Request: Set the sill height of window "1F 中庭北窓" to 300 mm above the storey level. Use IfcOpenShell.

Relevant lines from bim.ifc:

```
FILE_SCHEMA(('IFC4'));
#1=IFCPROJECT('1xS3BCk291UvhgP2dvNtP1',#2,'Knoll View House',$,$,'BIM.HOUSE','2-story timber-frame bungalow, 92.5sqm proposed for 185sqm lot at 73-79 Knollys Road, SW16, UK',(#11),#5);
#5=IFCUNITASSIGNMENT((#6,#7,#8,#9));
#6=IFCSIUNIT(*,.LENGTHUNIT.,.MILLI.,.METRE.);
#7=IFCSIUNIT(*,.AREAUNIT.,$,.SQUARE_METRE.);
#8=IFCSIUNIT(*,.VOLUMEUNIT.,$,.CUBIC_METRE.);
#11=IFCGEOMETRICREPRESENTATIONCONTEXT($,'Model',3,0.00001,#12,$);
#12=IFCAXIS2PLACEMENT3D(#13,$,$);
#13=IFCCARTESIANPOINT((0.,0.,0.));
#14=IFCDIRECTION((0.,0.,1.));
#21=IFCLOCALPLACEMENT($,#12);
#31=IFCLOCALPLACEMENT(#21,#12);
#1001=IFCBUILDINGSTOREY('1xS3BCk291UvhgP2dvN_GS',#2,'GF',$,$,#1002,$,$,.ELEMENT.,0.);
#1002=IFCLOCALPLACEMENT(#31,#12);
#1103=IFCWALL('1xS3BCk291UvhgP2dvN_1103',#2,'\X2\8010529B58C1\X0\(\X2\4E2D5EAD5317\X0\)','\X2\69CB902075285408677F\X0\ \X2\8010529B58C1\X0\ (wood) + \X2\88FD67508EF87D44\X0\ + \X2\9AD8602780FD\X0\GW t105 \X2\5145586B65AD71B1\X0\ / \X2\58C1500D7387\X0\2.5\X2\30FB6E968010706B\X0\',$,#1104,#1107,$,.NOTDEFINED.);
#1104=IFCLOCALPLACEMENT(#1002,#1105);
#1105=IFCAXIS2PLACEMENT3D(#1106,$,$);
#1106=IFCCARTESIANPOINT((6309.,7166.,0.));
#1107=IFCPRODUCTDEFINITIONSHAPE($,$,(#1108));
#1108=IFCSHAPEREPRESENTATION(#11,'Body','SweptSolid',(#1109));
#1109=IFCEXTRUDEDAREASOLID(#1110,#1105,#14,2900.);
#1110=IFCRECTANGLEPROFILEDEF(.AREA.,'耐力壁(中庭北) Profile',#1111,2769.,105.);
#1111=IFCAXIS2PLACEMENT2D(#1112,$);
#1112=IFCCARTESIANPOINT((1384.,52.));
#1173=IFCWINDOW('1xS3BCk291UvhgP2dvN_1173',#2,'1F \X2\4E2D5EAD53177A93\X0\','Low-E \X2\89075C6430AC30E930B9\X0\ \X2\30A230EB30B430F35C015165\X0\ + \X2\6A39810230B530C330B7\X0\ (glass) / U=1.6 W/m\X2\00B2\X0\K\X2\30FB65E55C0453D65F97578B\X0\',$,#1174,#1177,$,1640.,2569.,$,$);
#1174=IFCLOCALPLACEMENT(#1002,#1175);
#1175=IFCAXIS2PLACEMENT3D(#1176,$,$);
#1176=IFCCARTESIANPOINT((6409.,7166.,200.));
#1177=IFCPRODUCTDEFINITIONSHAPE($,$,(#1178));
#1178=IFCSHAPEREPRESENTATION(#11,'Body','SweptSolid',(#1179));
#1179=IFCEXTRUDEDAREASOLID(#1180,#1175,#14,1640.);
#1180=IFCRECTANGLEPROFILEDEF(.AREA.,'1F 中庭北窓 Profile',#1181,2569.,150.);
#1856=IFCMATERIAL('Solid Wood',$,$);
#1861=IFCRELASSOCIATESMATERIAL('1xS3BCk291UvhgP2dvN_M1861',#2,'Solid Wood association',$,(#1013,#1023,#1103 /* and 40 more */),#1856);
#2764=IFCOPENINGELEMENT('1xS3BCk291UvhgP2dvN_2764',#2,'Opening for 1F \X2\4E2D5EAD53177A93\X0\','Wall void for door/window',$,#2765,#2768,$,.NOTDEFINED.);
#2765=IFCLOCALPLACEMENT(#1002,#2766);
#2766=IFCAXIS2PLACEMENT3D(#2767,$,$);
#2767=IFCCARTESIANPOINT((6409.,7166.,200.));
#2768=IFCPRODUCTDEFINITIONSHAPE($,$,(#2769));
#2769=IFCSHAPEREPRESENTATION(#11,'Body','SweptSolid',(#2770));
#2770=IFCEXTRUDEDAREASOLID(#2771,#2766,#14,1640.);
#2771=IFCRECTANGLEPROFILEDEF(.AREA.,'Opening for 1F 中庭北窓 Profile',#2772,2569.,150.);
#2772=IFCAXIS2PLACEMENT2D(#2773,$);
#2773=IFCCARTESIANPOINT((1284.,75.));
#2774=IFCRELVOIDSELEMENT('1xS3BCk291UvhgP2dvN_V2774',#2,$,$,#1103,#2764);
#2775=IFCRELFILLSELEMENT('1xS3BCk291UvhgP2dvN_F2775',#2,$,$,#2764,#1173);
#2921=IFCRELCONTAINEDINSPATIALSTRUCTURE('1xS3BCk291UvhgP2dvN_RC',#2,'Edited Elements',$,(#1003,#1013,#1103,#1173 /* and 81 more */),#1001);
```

```python
import numpy as np
import ifcopenshell
import ifcopenshell.api.geometry
import ifcopenshell.geom
import ifcopenshell.util.element
import ifcopenshell.util.placement
import ifcopenshell.util.shape
import ifcopenshell.util.unit

model = ifcopenshell.open("bim.ifc")
unit_scale = ifcopenshell.util.unit.calculate_unit_scale(model)

window = model.by_guid("1xS3BCk291UvhgP2dvN_1173")
opening = window.FillsVoids[0].RelatingOpeningElement
storey = ifcopenshell.util.element.get_container(window, ifc_class="IfcBuildingStorey")
level = ifcopenshell.util.placement.get_local_placement(storey.ObjectPlacement)[2, 3]

# The opening's origin need not be at the sill, so measure its lowest point.
shape = ifcopenshell.geom.create_shape(ifcopenshell.geom.settings(), opening)
bottom = ifcopenshell.util.shape.get_shape_bottom_elevation(shape, shape.geometry) / unit_scale
dz = level + 300.0 - bottom

shift = np.array([0.0, 0.0, dz])
# The window is not placed relative to its opening, so move both.
for product in (opening, window):
    matrix = ifcopenshell.util.placement.get_local_placement(product.ObjectPlacement)
    matrix[:3, 3] += shift
    ifcopenshell.api.geometry.edit_object_placement(model, product=product, matrix=matrix, is_si=False)

print(f"moved by {dz * unit_scale:+.3f} m")

model.write("bim_v2.ifc")
```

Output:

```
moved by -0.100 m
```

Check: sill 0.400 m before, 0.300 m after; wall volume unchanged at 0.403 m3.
